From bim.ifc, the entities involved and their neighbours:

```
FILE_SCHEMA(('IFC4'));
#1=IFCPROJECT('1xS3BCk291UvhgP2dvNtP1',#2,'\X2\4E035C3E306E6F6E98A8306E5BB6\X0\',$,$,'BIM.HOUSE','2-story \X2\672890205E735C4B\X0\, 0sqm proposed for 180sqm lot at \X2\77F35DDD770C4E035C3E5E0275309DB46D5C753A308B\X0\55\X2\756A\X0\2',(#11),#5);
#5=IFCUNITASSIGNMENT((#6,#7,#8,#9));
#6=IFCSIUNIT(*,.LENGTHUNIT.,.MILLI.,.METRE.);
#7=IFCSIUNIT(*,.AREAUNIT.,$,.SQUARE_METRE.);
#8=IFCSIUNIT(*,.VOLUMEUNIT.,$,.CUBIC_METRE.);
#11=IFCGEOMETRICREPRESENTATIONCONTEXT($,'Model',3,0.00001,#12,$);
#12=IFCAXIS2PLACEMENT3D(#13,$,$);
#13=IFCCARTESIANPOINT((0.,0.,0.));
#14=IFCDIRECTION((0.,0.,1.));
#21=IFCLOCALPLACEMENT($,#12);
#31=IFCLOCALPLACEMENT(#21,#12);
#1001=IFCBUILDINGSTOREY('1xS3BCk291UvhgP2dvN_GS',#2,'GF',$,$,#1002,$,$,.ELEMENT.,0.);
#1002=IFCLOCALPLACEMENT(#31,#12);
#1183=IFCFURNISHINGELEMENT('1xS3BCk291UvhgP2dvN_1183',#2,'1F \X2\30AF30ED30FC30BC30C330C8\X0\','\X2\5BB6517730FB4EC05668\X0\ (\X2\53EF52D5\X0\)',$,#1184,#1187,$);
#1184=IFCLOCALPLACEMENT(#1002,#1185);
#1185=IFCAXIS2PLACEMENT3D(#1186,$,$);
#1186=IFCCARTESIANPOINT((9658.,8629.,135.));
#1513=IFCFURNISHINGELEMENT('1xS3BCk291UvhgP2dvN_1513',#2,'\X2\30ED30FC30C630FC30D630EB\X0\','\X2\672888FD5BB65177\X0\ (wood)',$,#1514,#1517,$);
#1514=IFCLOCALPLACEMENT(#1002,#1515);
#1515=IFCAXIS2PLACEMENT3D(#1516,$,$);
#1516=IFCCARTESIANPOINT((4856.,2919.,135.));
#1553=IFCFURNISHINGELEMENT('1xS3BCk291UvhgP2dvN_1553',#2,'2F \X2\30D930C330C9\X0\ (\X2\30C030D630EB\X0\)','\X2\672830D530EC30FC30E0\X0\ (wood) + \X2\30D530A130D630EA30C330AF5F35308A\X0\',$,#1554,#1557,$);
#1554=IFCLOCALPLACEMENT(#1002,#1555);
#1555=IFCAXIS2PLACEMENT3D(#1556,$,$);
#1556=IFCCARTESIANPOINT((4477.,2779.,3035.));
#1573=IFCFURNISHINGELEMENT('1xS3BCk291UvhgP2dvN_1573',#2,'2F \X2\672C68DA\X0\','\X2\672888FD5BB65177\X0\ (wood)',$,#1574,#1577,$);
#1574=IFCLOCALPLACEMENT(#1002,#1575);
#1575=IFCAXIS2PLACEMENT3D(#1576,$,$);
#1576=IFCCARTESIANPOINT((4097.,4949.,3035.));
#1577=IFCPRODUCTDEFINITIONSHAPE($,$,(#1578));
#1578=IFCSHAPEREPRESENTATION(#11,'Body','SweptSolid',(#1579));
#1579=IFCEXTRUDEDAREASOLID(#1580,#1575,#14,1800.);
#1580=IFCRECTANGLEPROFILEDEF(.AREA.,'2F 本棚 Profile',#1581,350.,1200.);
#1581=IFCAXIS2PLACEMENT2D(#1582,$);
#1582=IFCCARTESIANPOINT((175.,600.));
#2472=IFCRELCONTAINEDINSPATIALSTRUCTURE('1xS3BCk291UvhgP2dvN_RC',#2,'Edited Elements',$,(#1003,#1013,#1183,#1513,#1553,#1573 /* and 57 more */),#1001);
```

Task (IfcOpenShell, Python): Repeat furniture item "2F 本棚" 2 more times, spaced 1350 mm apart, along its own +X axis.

```python
import ifcopenshell
import ifcopenshell.api.geometry
import ifcopenshell.api.root
import ifcopenshell.util.element
import ifcopenshell.util.placement

model = ifcopenshell.open("bim.ifc")


def reuse_history(source, copy):
    """copy_class also copies each property set's owner history, people and application; keep the originals."""
    for rel in copy.IsDefinedBy:
        if rel.is_a("IfcRelDefinesByProperties") and (history := rel.RelatingPropertyDefinition.OwnerHistory):
            rel.RelatingPropertyDefinition.OwnerHistory = source.OwnerHistory
            ifcopenshell.util.element.remove_deep2(model, history)


source = model.by_guid("1xS3BCk291UvhgP2dvN_1573")
base = ifcopenshell.util.placement.get_local_placement(source.ObjectPlacement)
step = base[:3, 0] * 1350.0

for i in range(1, 3):
    copy = ifcopenshell.api.root.copy_class(model, product=source)
    copy.Representation = ifcopenshell.util.element.copy_deep(
        model, source.Representation, exclude=["IfcGeometricRepresentationContext", "IfcRepresentationMap"]
    )
    reuse_history(source, copy)
    matrix = base.copy()
    matrix[:3, 3] += i * step
    print("added at", matrix[:3, 3].round(3) + 0.0)
    ifcopenshell.api.geometry.edit_object_placement(model, product=copy, matrix=matrix, is_si=False)

model.write("bim_updated.ifc")
```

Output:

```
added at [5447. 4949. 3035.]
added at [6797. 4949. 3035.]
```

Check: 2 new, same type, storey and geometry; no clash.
